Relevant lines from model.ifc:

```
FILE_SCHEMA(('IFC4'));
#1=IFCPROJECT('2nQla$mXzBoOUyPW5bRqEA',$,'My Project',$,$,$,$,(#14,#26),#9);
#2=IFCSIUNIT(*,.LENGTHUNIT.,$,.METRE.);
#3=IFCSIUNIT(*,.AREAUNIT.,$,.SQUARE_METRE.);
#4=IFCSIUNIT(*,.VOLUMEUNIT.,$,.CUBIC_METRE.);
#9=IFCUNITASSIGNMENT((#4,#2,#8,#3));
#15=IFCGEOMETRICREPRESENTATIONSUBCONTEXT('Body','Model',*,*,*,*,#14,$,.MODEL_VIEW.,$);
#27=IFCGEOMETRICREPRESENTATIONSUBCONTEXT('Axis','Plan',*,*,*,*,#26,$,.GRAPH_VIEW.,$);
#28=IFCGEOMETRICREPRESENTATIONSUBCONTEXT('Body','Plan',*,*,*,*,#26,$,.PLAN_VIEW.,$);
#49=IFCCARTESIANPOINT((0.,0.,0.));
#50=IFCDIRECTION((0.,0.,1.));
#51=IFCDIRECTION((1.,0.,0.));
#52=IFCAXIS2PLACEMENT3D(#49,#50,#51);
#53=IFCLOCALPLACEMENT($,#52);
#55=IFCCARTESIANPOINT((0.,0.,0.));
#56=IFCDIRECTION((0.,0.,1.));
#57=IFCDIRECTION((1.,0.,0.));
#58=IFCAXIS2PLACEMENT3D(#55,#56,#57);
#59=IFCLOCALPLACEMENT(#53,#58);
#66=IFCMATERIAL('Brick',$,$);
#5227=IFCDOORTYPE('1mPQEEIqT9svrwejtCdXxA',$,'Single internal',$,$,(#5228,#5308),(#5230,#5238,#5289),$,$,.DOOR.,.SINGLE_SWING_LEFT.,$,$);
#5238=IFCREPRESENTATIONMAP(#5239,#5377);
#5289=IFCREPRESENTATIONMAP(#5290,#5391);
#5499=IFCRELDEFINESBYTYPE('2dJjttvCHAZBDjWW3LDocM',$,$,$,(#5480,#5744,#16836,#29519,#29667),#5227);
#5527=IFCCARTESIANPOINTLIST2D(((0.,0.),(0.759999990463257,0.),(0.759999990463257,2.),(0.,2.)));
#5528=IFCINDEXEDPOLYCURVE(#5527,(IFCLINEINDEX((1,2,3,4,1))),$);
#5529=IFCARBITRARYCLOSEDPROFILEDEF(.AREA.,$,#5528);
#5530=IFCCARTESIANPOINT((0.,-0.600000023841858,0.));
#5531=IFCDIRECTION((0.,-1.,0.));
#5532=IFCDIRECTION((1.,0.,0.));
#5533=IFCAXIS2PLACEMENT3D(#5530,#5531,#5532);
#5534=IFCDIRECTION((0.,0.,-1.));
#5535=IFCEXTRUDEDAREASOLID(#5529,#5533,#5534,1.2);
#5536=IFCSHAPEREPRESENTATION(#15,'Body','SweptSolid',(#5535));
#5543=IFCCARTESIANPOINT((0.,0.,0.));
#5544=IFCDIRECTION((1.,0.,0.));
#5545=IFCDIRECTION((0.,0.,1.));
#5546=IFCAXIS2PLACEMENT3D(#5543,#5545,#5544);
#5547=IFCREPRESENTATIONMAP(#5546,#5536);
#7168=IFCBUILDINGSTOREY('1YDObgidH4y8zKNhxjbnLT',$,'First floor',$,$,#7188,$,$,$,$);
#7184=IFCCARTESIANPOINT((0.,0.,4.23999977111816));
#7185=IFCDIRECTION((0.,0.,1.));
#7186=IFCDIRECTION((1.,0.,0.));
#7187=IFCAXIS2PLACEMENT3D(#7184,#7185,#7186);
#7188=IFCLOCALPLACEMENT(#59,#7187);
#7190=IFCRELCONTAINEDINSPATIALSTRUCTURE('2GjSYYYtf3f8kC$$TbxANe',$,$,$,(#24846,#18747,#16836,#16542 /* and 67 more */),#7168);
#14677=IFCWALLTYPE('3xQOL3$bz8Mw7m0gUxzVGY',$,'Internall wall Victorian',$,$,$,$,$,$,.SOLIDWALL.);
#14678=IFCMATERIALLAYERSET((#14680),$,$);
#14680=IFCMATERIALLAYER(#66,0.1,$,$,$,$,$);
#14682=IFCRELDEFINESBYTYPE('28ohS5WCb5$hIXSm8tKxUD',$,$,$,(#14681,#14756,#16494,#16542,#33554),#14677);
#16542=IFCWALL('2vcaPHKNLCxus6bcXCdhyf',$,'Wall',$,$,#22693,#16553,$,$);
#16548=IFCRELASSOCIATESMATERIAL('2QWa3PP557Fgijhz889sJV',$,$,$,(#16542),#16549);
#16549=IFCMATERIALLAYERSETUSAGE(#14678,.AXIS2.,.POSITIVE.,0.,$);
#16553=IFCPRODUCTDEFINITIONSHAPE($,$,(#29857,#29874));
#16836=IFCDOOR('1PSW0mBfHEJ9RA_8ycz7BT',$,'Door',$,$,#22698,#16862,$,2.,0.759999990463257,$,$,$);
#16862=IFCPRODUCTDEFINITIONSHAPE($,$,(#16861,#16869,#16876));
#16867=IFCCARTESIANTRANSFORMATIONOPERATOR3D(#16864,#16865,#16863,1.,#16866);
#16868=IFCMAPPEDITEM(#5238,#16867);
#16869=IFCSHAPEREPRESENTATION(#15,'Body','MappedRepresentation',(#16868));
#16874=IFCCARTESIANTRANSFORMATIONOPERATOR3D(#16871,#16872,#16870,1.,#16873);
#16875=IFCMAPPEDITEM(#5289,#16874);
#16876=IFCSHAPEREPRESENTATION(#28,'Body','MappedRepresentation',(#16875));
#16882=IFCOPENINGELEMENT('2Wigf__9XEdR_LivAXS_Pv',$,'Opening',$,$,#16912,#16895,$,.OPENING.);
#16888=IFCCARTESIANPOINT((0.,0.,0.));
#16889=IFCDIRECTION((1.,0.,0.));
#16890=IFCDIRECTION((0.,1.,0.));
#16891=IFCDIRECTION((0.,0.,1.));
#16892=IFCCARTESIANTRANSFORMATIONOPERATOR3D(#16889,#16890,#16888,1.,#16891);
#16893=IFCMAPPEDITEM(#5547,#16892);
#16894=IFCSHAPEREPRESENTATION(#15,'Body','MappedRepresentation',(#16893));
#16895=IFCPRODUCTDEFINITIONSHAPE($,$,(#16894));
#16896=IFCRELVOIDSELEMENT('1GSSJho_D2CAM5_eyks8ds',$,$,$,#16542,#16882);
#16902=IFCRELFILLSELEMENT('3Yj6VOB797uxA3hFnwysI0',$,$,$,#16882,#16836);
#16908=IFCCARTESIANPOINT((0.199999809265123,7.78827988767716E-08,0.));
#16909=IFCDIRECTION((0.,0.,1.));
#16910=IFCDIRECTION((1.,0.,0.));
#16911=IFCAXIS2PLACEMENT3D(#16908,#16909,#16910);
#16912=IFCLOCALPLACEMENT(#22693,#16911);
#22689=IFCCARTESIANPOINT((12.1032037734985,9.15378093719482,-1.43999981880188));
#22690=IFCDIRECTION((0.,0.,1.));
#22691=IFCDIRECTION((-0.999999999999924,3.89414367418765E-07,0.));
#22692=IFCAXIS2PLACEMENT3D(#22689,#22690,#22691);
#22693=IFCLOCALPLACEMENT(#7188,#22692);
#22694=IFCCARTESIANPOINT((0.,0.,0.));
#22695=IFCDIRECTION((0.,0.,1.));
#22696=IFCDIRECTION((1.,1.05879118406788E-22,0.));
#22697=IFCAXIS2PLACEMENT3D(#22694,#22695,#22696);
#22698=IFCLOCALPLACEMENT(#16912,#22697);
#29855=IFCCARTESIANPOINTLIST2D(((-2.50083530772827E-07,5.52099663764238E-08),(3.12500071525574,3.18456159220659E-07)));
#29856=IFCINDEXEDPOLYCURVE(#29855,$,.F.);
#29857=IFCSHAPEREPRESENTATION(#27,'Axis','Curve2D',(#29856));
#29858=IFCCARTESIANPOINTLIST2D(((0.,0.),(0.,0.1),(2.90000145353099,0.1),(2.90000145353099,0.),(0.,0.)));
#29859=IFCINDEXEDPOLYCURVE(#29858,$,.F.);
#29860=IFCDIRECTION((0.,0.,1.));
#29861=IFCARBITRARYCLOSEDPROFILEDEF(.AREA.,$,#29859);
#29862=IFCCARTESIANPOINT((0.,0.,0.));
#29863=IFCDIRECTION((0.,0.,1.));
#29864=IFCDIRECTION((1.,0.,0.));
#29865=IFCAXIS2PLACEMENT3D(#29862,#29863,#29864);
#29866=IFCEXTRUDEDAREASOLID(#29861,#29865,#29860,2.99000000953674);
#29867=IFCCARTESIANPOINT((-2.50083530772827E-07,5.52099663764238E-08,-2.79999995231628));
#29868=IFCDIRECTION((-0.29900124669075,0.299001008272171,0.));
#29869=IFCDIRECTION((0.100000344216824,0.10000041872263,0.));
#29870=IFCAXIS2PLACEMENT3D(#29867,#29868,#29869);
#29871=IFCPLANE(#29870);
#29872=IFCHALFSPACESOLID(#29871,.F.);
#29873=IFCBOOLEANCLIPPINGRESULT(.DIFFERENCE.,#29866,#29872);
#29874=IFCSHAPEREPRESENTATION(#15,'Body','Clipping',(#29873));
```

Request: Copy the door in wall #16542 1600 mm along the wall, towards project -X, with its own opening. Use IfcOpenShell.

```python
import ifcopenshell
import ifcopenshell.api.feature
import ifcopenshell.api.geometry
import ifcopenshell.api.root
import ifcopenshell.geom
import ifcopenshell.util.element
import ifcopenshell.util.placement
import ifcopenshell.util.shape

model = ifcopenshell.open("model.ifc")
settings = ifcopenshell.geom.settings()


def volume(element):
    """Net volume in cubic metres, openings subtracted."""
    shape = ifcopenshell.geom.create_shape(settings, element)
    return ifcopenshell.util.shape.get_volume(shape.geometry)


door = model.by_id(16836)
opening = door.FillsVoids[0].RelatingOpeningElement
wall = opening.VoidsElements[0].RelatingBuildingElement
before = volume(wall)
shift = ifcopenshell.util.placement.get_local_placement(wall.ObjectPlacement)[:3, 0] * 1.6

# copy_class copies the void relationship, type, container and properties, but no geometry.
new_opening = ifcopenshell.api.root.copy_class(model, product=opening)
new_opening.Representation = ifcopenshell.util.element.copy_deep(
    model, opening.Representation, exclude=["IfcGeometricRepresentationContext", "IfcRepresentationMap"]
)
new_door = ifcopenshell.api.root.copy_class(model, product=door)
new_door.Representation = ifcopenshell.util.element.copy_deep(
    model, door.Representation, exclude=["IfcGeometricRepresentationContext", "IfcRepresentationMap"]
)
ifcopenshell.api.feature.add_filling(model, opening=new_opening, element=new_door)

for old, new in ((opening, new_opening), (door, new_door)):
    matrix = ifcopenshell.util.placement.get_local_placement(old.ObjectPlacement)
    matrix[:3, 3] += shift
    ifcopenshell.api.geometry.edit_object_placement(model, product=new, matrix=matrix, is_si=False)

after = volume(wall)

print(f"wall volume {before:.3f} -> {after:.3f} m3")

model.write("model_v2.ifc")
```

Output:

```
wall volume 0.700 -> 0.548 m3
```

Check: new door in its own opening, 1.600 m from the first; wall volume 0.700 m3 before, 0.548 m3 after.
